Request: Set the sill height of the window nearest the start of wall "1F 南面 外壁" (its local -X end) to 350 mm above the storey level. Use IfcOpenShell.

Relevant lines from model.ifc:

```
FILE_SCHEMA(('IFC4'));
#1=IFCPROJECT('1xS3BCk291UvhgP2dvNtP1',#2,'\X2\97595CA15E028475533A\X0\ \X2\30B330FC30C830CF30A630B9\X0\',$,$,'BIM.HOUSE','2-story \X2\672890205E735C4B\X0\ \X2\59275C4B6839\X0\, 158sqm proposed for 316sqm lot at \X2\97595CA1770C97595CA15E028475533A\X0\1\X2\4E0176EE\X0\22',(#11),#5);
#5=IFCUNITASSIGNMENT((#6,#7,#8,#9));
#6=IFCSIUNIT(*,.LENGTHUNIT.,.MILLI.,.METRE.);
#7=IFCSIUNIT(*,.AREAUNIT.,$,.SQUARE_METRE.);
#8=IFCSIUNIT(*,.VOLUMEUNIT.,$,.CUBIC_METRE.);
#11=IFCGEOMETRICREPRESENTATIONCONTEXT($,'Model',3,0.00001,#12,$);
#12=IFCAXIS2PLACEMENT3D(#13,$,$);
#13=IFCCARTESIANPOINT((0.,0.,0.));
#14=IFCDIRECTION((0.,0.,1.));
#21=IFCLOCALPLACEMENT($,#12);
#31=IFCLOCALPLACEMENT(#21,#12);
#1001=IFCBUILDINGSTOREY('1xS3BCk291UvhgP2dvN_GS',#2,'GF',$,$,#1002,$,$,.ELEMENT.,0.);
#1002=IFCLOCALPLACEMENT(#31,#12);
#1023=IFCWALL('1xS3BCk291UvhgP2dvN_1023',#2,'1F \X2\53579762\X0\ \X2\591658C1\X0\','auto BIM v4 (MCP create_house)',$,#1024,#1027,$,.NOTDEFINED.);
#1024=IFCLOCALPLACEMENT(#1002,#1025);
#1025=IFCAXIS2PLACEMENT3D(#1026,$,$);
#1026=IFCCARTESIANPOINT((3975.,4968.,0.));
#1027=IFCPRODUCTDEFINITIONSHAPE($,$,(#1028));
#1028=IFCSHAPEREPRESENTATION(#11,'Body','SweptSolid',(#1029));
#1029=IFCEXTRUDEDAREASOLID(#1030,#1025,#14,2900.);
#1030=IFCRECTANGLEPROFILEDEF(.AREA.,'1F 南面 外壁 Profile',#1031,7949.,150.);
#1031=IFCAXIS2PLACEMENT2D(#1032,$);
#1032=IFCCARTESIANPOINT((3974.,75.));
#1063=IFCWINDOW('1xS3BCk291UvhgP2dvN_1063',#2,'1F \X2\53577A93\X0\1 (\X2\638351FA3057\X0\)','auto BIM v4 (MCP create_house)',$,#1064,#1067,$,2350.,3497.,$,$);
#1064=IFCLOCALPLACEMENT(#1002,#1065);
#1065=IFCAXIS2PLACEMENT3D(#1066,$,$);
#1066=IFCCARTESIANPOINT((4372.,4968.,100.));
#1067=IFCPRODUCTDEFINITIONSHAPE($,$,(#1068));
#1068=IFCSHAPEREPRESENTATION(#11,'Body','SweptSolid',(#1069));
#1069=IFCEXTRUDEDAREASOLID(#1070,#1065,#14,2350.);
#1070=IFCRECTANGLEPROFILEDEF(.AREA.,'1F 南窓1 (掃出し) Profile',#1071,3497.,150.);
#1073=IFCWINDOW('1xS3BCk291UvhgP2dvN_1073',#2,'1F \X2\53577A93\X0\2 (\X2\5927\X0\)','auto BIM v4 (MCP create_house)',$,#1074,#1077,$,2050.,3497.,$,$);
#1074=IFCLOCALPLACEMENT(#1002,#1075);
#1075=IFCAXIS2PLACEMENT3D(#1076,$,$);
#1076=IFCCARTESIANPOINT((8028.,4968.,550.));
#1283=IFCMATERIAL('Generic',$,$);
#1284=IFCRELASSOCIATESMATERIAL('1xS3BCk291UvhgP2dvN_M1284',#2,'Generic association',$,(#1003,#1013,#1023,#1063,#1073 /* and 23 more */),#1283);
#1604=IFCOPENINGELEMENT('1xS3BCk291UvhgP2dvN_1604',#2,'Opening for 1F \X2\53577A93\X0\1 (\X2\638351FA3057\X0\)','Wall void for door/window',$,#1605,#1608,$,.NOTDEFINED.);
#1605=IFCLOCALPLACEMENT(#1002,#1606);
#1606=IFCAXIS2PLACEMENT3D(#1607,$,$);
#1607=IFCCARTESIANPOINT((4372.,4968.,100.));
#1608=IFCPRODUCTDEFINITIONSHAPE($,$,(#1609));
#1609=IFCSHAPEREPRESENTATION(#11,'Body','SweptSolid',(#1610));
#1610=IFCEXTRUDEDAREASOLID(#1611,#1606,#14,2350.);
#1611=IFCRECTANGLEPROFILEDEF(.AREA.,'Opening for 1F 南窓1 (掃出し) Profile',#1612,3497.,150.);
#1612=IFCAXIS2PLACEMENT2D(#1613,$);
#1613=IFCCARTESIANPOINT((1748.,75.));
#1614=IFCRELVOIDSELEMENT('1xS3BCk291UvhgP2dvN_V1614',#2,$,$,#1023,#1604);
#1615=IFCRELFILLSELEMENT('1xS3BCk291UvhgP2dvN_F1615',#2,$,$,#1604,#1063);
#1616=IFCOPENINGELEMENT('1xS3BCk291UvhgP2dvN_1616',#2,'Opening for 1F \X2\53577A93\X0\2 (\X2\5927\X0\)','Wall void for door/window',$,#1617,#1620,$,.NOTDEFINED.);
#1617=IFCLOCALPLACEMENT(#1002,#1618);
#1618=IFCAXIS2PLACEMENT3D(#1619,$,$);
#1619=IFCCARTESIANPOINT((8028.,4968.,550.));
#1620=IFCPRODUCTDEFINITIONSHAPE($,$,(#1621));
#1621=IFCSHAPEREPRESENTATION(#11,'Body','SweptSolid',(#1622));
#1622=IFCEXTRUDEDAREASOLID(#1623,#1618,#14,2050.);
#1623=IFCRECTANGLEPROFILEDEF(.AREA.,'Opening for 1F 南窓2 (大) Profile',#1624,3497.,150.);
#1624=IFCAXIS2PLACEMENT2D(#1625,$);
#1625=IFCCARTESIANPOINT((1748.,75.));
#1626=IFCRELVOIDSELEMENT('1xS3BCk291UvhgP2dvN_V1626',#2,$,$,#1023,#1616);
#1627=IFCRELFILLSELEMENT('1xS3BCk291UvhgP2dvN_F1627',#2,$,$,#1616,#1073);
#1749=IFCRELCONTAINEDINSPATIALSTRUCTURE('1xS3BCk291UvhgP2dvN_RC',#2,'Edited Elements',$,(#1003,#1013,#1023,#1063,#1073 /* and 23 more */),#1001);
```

```python
import numpy as np
import ifcopenshell
import ifcopenshell.api.geometry
import ifcopenshell.geom
import ifcopenshell.util.element
import ifcopenshell.util.placement
import ifcopenshell.util.shape
import ifcopenshell.util.unit

model = ifcopenshell.open("model.ifc")
unit_scale = ifcopenshell.util.unit.calculate_unit_scale(model)

window = model.by_id(1063)
opening = window.FillsVoids[0].RelatingOpeningElement
storey = ifcopenshell.util.element.get_container(window, ifc_class="IfcBuildingStorey")
level = ifcopenshell.util.placement.get_local_placement(storey.ObjectPlacement)[2, 3]

# The opening's origin need not be at the sill, so measure its lowest point.
shape = ifcopenshell.geom.create_shape(ifcopenshell.geom.settings(), opening)
bottom = ifcopenshell.util.shape.get_shape_bottom_elevation(shape, shape.geometry) / unit_scale
dz = level + 0.35 / unit_scale - bottom

shift = np.array([0.0, 0.0, dz])
# The window is not placed relative to its opening, so move both.
for product in (opening, window):
    matrix = ifcopenshell.util.placement.get_local_placement(product.ObjectPlacement)
    matrix[:3, 3] += shift
    ifcopenshell.api.geometry.edit_object_placement(model, product=product, matrix=matrix, is_si=False)

print(f"moved by {dz * unit_scale:+.3f} m")

model.write("model_v2.ifc")
```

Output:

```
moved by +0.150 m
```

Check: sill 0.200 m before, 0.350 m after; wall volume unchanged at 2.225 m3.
